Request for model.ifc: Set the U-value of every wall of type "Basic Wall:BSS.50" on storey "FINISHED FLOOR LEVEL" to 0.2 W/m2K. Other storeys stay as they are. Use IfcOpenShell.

First a look at what the model holds.

```python
import ifcopenshell
import ifcopenshell.util.element

model = ifcopenshell.open("model.ifc")
print(model.schema)
storey = next(s for s in model.by_type("IfcBuildingStorey") if s.Name == "FINISHED FLOOR LEVEL")
walls = [e for e in ifcopenshell.util.element.get_decomposition(storey) if e.is_a("IfcWall")]
seen = {}
for e in walls:
    element_type = ifcopenshell.util.element.get_type(e)
    key = (element_type.Name if element_type != e and element_type else None, ifcopenshell.util.element.get_pset(e, "Pset_WallCommon", "ThermalTransmittance"))
    seen[key] = seen.get(key, 0) + 1
for (name, value), count in sorted(seen.items(), key=str):
    print(count, "x", name, "|", value)
```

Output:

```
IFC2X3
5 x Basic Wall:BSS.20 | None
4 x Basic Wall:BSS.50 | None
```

```python
import ifcopenshell
import ifcopenshell.api.pset
import ifcopenshell.util.element

model = ifcopenshell.open("model.ifc")

storey = next(s for s in model.by_type("IfcBuildingStorey") if s.Name == "FINISHED FLOOR LEVEL")
walls = [e for e in ifcopenshell.util.element.get_decomposition(storey) if e.is_a("IfcWall")]

count = 0
for e in walls:
    element_type = ifcopenshell.util.element.get_type(e)
    if element_type in (None, e) or element_type.Name != "Basic Wall:BSS.50":
        continue
    # add_pset returns the element's existing set when there is one.
    pset = ifcopenshell.api.pset.add_pset(model, product=e, name="Pset_WallCommon")
    ifcopenshell.api.pset.edit_pset(model, pset=pset, properties={"ThermalTransmittance": 0.2})
    count += 1

print(count, "walls updated")

model.write("model-out.ifc")
```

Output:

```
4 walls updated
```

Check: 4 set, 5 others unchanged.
